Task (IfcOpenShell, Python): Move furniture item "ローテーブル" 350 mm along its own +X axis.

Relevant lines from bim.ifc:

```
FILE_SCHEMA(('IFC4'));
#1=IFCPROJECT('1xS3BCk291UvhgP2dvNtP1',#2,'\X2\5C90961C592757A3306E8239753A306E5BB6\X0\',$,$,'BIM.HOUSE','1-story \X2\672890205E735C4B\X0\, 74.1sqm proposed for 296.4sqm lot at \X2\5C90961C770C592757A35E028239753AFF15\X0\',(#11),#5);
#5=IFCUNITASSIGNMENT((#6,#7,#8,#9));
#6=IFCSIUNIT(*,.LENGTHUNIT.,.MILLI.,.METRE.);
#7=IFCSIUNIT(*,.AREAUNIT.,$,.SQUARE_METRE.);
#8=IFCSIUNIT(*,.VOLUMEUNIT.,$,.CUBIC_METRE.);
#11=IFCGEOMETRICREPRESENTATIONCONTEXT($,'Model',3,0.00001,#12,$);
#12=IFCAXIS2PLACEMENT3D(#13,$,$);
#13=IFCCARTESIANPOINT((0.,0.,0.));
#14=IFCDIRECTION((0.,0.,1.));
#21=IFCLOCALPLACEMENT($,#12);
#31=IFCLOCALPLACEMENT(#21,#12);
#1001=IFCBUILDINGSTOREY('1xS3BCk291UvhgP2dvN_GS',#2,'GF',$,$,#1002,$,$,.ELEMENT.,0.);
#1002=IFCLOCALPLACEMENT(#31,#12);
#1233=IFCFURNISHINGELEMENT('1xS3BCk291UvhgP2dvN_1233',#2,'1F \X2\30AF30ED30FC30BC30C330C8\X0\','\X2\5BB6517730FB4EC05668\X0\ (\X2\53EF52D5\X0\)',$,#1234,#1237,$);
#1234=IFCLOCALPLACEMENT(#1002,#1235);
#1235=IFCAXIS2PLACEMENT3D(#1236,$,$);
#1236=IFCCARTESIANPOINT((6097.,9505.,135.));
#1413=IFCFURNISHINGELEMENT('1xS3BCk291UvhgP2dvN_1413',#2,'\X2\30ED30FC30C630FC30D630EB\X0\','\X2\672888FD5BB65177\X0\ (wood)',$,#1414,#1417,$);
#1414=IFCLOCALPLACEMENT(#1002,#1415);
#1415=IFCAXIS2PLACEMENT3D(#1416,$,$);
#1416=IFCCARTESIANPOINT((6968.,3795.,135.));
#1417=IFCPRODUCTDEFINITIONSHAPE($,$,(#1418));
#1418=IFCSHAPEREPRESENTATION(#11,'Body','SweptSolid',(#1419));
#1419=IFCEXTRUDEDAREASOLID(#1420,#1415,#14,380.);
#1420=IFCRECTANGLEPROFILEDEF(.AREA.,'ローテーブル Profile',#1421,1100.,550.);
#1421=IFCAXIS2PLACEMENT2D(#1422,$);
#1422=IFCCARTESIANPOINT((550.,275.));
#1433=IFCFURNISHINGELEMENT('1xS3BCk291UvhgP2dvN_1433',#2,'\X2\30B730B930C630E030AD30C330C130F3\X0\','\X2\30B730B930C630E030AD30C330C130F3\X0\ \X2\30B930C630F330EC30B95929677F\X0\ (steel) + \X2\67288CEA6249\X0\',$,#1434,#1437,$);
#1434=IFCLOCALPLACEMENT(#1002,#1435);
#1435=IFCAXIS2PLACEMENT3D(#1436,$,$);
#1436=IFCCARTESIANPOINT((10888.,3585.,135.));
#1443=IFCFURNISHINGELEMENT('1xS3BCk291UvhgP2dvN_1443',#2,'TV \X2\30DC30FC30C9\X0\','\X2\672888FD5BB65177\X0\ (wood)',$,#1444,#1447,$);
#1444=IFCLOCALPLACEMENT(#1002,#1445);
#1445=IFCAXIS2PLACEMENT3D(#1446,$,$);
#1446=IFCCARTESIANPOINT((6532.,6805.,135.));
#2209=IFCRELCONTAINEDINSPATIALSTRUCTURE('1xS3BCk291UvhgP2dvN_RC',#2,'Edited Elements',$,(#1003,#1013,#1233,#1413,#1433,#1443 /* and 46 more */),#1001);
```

```python
import ifcopenshell
import ifcopenshell.api.geometry
import ifcopenshell.util.placement
import ifcopenshell.util.unit

model = ifcopenshell.open("bim.ifc")
unit_scale = ifcopenshell.util.unit.calculate_unit_scale(model)

item = model.by_guid("1xS3BCk291UvhgP2dvN_1413")
matrix = ifcopenshell.util.placement.get_local_placement(item.ObjectPlacement)
matrix[:3, 3] += matrix[:3, 0] * 0.35 / unit_scale
ifcopenshell.api.geometry.edit_object_placement(model, product=item, matrix=matrix, is_si=False)

print(ifcopenshell.util.placement.get_local_placement(item.ObjectPlacement).round(3) + 0.0)

model.write("bim_rev.ifc")
```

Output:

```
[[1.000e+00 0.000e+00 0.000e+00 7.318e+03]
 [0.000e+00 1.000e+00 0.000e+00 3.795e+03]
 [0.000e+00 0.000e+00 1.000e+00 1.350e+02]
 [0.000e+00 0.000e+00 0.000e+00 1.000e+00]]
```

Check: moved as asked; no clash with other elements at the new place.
